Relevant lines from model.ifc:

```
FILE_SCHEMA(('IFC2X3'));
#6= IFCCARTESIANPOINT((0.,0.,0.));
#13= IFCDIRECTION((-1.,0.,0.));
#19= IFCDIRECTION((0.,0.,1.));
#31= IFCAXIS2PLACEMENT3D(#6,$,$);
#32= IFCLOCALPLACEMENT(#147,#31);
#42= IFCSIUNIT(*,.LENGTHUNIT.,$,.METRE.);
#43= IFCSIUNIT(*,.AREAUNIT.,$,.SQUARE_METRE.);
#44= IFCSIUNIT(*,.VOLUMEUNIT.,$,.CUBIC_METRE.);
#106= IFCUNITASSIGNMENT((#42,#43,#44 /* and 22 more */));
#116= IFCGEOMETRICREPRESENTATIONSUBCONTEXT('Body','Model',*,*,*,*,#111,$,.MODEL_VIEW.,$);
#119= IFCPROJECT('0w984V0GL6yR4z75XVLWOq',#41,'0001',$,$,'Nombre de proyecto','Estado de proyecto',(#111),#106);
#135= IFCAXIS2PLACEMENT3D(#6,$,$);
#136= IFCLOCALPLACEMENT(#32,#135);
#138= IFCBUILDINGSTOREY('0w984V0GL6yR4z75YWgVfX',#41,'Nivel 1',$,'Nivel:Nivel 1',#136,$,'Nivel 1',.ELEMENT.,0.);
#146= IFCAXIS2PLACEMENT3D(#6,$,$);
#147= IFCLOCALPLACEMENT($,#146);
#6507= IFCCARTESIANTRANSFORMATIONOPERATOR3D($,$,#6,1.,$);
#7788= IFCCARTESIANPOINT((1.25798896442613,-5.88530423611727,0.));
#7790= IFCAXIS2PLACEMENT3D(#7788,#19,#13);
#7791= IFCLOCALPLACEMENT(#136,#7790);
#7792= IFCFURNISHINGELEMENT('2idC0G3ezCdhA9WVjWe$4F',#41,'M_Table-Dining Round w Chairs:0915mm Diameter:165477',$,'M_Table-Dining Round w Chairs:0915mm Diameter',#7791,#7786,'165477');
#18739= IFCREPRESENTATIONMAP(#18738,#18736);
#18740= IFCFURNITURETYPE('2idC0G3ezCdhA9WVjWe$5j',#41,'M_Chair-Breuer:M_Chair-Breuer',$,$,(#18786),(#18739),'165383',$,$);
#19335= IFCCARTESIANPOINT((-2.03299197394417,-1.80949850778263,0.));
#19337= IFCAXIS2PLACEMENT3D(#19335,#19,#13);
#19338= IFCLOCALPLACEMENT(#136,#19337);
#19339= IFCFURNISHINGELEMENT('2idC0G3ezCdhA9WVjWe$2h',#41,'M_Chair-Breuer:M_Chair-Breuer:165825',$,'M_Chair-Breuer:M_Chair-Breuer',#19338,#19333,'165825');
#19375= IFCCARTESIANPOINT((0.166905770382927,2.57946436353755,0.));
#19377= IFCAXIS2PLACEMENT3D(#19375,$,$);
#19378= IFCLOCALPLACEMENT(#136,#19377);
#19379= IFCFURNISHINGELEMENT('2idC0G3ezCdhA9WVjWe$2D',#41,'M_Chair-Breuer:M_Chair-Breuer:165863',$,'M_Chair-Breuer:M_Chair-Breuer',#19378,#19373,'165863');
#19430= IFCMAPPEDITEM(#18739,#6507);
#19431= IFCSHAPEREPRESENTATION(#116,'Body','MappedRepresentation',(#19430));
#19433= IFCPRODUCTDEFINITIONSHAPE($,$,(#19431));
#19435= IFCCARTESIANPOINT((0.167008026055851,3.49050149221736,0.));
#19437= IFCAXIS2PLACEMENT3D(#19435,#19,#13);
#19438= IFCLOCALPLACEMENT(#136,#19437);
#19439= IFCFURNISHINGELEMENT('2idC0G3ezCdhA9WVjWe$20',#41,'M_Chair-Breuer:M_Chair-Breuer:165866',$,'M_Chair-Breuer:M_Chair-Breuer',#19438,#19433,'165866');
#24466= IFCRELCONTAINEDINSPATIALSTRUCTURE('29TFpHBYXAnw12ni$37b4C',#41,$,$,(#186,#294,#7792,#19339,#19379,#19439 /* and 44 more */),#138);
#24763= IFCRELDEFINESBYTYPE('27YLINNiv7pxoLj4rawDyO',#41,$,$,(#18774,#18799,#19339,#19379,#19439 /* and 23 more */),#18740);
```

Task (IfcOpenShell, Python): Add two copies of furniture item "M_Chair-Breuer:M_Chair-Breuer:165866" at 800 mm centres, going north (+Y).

```python
import numpy as np
import ifcopenshell
import ifcopenshell.api.geometry
import ifcopenshell.api.root
import ifcopenshell.util.element
import ifcopenshell.util.placement
import ifcopenshell.util.unit

model = ifcopenshell.open("model.ifc")
unit_scale = ifcopenshell.util.unit.calculate_unit_scale(model)


def reuse_history(source, copy):
    """copy_class also copies each property set's owner history, people and application; keep the originals."""
    for rel in copy.IsDefinedBy:
        if rel.is_a("IfcRelDefinesByProperties") and (history := rel.RelatingPropertyDefinition.OwnerHistory):
            rel.RelatingPropertyDefinition.OwnerHistory = source.OwnerHistory
            ifcopenshell.util.element.remove_deep2(model, history)


source = model.by_id(19439)
base = ifcopenshell.util.placement.get_local_placement(source.ObjectPlacement)
step = np.array([0.0, 1.0, 0.0]) * 0.8 / unit_scale

for i in range(1, 3):
    copy = ifcopenshell.api.root.copy_class(model, product=source)
    copy.Representation = ifcopenshell.util.element.copy_deep(
        model, source.Representation, exclude=["IfcGeometricRepresentationContext", "IfcRepresentationMap"]
    )
    copy.Name = "M_Chair-Breuer:M_Chair-Breuer"
    copy.Tag = None
    reuse_history(source, copy)
    matrix = base.copy()
    matrix[:3, 3] += i * step
    print("added at", matrix[:3, 3].round(3) + 0.0)
    ifcopenshell.api.geometry.edit_object_placement(model, product=copy, matrix=matrix, is_si=False)

model.write("model_updated.ifc")
```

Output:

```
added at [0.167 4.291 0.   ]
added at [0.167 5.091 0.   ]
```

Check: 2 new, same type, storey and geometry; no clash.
